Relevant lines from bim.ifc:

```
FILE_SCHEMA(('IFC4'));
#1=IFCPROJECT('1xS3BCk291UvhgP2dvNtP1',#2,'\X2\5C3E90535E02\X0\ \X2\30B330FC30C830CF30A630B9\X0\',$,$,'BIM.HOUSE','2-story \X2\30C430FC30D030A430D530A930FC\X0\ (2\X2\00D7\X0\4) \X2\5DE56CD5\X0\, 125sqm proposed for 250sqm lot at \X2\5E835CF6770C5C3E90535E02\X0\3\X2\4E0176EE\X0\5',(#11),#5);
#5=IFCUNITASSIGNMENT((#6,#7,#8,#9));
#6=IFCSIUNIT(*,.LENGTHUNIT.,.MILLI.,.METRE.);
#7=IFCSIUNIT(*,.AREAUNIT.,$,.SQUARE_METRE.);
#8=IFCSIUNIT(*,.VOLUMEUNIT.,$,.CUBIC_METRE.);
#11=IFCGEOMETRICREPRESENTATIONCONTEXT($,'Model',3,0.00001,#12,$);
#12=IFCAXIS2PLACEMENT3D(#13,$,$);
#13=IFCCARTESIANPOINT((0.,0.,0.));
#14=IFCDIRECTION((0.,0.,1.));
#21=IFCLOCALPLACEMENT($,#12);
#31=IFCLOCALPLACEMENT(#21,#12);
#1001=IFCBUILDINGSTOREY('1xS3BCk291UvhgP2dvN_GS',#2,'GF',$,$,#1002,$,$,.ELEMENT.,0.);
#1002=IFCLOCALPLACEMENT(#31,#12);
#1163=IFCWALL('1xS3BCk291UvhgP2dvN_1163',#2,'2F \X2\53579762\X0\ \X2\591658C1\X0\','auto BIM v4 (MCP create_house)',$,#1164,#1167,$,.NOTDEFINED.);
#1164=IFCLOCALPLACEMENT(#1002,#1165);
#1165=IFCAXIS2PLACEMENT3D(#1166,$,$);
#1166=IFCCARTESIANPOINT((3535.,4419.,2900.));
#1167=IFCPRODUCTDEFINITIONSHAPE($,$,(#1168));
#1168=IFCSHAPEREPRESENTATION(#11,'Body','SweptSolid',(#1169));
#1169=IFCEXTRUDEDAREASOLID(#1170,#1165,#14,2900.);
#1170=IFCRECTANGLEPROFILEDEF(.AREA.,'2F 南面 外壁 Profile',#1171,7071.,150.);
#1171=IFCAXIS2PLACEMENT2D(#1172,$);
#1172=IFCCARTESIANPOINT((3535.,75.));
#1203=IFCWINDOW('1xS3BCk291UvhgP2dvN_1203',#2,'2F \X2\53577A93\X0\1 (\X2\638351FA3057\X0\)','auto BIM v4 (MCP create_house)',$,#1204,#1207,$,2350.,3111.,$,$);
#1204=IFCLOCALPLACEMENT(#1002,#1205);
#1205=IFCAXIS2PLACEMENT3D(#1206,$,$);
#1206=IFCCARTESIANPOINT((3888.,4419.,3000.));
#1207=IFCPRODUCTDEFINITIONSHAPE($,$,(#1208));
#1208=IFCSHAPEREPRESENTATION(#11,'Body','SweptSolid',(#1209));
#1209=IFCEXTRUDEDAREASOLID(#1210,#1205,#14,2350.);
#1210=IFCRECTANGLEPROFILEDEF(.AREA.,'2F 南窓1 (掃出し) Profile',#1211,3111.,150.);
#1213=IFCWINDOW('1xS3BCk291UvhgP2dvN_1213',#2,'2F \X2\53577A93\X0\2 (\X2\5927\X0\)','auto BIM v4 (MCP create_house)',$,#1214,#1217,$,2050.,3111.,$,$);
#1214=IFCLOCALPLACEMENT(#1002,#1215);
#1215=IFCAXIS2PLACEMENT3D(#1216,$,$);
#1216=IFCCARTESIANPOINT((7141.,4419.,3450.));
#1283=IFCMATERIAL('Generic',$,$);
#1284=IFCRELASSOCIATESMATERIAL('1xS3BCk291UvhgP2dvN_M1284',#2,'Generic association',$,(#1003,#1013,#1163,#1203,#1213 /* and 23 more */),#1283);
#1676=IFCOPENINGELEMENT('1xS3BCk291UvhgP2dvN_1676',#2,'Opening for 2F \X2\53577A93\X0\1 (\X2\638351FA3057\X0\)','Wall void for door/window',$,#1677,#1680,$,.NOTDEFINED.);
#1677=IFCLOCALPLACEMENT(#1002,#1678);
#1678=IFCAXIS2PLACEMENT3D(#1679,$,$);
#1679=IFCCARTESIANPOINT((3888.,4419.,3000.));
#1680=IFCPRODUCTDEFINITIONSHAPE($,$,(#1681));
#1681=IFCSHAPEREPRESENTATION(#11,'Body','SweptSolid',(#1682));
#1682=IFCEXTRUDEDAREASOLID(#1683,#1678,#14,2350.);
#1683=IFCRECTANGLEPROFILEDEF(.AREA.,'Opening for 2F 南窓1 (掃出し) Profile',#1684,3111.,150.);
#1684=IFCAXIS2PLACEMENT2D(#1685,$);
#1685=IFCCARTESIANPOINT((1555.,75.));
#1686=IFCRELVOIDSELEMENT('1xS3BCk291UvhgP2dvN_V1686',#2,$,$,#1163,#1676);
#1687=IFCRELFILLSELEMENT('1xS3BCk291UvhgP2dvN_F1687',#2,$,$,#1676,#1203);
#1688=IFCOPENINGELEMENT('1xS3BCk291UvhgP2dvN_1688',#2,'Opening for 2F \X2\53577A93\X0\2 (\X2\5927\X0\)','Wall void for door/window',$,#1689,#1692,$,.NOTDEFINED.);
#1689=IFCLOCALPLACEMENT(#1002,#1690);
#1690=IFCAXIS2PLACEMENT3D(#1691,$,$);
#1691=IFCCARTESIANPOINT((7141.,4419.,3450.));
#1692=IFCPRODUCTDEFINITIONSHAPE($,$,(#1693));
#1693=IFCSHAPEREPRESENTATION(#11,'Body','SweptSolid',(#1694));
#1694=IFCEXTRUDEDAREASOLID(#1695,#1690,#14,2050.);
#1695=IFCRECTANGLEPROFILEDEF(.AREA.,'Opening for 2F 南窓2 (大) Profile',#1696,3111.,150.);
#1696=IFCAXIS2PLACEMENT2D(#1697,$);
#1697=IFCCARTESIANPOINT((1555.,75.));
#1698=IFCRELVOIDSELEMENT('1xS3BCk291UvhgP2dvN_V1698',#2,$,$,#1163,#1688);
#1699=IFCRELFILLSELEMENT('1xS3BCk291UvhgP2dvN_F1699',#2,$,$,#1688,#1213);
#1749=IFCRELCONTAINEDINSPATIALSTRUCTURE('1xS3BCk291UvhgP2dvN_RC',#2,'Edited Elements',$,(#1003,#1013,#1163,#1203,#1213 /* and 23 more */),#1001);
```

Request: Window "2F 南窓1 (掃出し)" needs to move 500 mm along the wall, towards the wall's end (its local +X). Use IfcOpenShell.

```python
import ifcopenshell
import ifcopenshell.api.geometry
import ifcopenshell.util.placement
import ifcopenshell.util.unit

model = ifcopenshell.open("bim.ifc")
unit_scale = ifcopenshell.util.unit.calculate_unit_scale(model)

window = model.by_guid("1xS3BCk291UvhgP2dvN_1203")
opening = window.FillsVoids[0].RelatingOpeningElement
wall = opening.VoidsElements[0].RelatingBuildingElement

wall_matrix = ifcopenshell.util.placement.get_local_placement(wall.ObjectPlacement)
shift = wall_matrix[:3, 0] * 0.5 / unit_scale
before = ifcopenshell.util.placement.get_local_placement(window.ObjectPlacement)[:3, 3].copy()

# The window is not placed relative to its opening, so move both.
for product in (opening, window):
    matrix = ifcopenshell.util.placement.get_local_placement(product.ObjectPlacement)
    matrix[:3, 3] += shift
    ifcopenshell.api.geometry.edit_object_placement(model, product=product, matrix=matrix, is_si=False)

after = ifcopenshell.util.placement.get_local_placement(window.ObjectPlacement)[:3, 3]
print("window moved by", (after - before).round(3) + 0.0)

model.write("bim_updated.ifc")
```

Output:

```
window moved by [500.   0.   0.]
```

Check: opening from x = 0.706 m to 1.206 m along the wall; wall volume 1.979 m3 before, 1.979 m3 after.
